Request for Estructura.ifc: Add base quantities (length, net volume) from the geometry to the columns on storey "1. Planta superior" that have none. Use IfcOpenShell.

First a look at what the model holds.

```python
import ifcopenshell
import ifcopenshell.util.element
import ifcopenshell.util.unit

model = ifcopenshell.open("Estructura.ifc")
print(model.schema)
for unit_type in ("LENGTHUNIT", "AREAUNIT", "VOLUMEUNIT"):
    print(unit_type, ifcopenshell.util.unit.calculate_unit_scale(model, unit_type))
storey = next(s for s in model.by_type("IfcBuildingStorey") if s.Name == "1. Planta superior")
columns = [e for e in ifcopenshell.util.element.get_decomposition(storey) if e.is_a("IfcColumn")]
for e in sorted(columns, key=lambda e: e.id()):
    print(e.id(), e.is_a(), e.Name, list(ifcopenshell.util.element.get_psets(e, qtos_only=True)), sep=" | ")
```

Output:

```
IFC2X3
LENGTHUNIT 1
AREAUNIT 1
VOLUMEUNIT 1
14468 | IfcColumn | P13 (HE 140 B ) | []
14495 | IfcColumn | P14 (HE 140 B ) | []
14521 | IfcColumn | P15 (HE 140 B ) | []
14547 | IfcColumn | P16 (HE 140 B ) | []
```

```python
import ifcopenshell
import ifcopenshell.api.pset
import ifcopenshell.geom
import ifcopenshell.util.element
import ifcopenshell.util.shape
import ifcopenshell.util.unit

model = ifcopenshell.open("Estructura.ifc")
unit_scale = ifcopenshell.util.unit.calculate_unit_scale(model)
volume_scale = ifcopenshell.util.unit.calculate_unit_scale(model, "VOLUMEUNIT")
settings = ifcopenshell.geom.settings()

storey = next(s for s in model.by_type("IfcBuildingStorey") if s.Name == "1. Planta superior")
columns = [e for e in ifcopenshell.util.element.get_decomposition(storey) if e.is_a("IfcColumn")]

for e in sorted(columns, key=lambda e: e.id()):
    if ifcopenshell.util.element.get_psets(e, qtos_only=True, should_inherit=False):
        continue
    # Geometry comes back in metres, in the element's own axes.
    shape = ifcopenshell.geom.create_shape(settings, e)
    values = {
        "Length": ifcopenshell.util.shape.get_z(shape.geometry) / unit_scale,
        "NetVolume": ifcopenshell.util.shape.get_volume(shape.geometry) / volume_scale,
    }
    qto = ifcopenshell.api.pset.add_qto(model, product=e, name="BaseQuantities")
    ifcopenshell.api.pset.edit_qto(model, qto=qto, properties=values)
    print(e.id(), {k: round(v, 3) for k, v in values.items()})

model.write("Estructura_v2.ifc")
```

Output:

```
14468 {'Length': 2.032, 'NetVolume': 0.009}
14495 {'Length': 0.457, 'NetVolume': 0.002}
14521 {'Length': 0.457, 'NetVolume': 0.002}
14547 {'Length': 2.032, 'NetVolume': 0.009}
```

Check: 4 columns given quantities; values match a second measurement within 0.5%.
